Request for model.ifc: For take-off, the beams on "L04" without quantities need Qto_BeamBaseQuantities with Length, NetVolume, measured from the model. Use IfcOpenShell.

First a look at what the model holds.

```python
import ifcopenshell
import ifcopenshell.util.element
import ifcopenshell.util.unit

model = ifcopenshell.open("model.ifc")
print(model.schema)
for unit_type in ("LENGTHUNIT", "AREAUNIT", "VOLUMEUNIT"):
    print(unit_type, ifcopenshell.util.unit.calculate_unit_scale(model, unit_type))
storey = next(s for s in model.by_type("IfcBuildingStorey") if s.Name == "L04")
beams = [e for e in ifcopenshell.util.element.get_decomposition(storey) if e.is_a("IfcBeam")]
for e in sorted(beams, key=lambda e: e.id()):
    print(e.id(), e.is_a(), e.Name, list(ifcopenshell.util.element.get_psets(e, qtos_only=True)), sep=" | ")
```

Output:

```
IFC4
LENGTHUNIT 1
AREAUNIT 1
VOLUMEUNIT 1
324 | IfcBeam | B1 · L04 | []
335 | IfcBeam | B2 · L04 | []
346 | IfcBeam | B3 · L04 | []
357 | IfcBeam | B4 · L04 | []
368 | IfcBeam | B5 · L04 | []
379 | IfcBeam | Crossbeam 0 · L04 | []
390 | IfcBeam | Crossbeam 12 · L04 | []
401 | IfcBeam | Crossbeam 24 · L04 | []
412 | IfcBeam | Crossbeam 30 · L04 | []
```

```python
import ifcopenshell
import ifcopenshell.api.pset
import ifcopenshell.geom
import ifcopenshell.util.element
import ifcopenshell.util.shape
import ifcopenshell.util.unit

model = ifcopenshell.open("model.ifc")
unit_scale = ifcopenshell.util.unit.calculate_unit_scale(model)
volume_scale = ifcopenshell.util.unit.calculate_unit_scale(model, "VOLUMEUNIT")
settings = ifcopenshell.geom.settings()

storey = next(s for s in model.by_type("IfcBuildingStorey") if s.Name == "L04")
beams = [e for e in ifcopenshell.util.element.get_decomposition(storey) if e.is_a("IfcBeam")]

for e in sorted(beams, key=lambda e: e.id()):
    if ifcopenshell.util.element.get_psets(e, qtos_only=True, should_inherit=False):
        continue
    # Geometry comes back in metres, in the element's own axes.
    shape = ifcopenshell.geom.create_shape(settings, e)
    values = {
        "Length": ifcopenshell.util.shape.get_max_xyz(shape.geometry) / unit_scale,
        "NetVolume": ifcopenshell.util.shape.get_volume(shape.geometry) / volume_scale,
    }
    qto = ifcopenshell.api.pset.add_qto(model, product=e, name="Qto_BeamBaseQuantities")
    ifcopenshell.api.pset.edit_qto(model, qto=qto, properties=values)
    print(e.id(), {k: round(v, 3) for k, v in values.items()})

model.write("model-out.ifc")
```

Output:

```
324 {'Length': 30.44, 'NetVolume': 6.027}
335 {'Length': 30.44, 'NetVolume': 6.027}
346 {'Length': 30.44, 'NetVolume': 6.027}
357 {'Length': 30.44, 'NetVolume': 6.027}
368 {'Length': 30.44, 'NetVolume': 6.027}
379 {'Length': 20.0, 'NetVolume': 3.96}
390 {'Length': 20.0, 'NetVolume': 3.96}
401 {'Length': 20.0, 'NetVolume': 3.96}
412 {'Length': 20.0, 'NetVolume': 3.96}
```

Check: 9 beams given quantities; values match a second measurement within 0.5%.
